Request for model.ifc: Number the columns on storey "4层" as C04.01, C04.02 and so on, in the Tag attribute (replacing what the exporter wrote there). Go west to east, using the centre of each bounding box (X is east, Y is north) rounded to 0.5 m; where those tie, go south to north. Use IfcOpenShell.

First a look at what the model holds.

```python
import ifcopenshell
import ifcopenshell.util.element
import ifcopenshell.util.placement

model = ifcopenshell.open("model.ifc")
print(model.schema)
storey = next(s for s in model.by_type("IfcBuildingStorey") if s.Name == "4层")
columns = [e for e in ifcopenshell.util.element.get_decomposition(storey) if e.is_a("IfcColumn")]
for e in sorted(columns, key=lambda e: e.id()):
    origin = ifcopenshell.util.placement.get_local_placement(e.ObjectPlacement)[:3, 3]
    print(e.id(), e.Tag, e.Name, origin.round(2) + 0.0, sep=" | ")
```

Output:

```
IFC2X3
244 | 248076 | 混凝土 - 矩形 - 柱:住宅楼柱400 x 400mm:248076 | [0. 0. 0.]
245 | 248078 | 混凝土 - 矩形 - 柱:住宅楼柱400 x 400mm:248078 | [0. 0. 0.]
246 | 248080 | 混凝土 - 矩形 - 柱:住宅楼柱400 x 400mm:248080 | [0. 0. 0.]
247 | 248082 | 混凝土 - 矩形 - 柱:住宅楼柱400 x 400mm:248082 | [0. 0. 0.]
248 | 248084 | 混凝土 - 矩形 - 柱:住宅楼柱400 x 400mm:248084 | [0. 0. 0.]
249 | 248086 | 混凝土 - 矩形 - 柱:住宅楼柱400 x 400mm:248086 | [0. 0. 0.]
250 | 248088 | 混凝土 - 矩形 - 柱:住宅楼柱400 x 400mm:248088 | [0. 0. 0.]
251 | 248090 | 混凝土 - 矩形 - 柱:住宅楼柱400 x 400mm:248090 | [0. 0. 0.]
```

```python
import ifcopenshell
import ifcopenshell.geom
import ifcopenshell.util.element
import ifcopenshell.util.shape

model = ifcopenshell.open("model.ifc")
settings = ifcopenshell.geom.settings()
settings.set("use-world-coords", True)


def centre(element):
    shape = ifcopenshell.geom.create_shape(settings, element)
    return ifcopenshell.util.shape.get_bbox_centroid(shape.geometry)


storey = next(s for s in model.by_type("IfcBuildingStorey") if s.Name == "4层")
columns = [e for e in ifcopenshell.util.element.get_decomposition(storey) if e.is_a("IfcColumn")]

# Insertion points can sit at a corner or the storey origin, so sort by the geometry (in metres).
centres = {e: centre(e) for e in columns}
columns.sort(key=lambda e: (round(centres[e][0] / 0.5), centres[e][1]))

for i, e in enumerate(columns, start=1):
    number = f"C04.{i:02d}"
    e.Tag = number
    print(e.id(), number)

model.write("model_v2.ifc")
```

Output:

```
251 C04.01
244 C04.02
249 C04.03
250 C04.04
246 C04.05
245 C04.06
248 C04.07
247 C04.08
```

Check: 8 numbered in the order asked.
